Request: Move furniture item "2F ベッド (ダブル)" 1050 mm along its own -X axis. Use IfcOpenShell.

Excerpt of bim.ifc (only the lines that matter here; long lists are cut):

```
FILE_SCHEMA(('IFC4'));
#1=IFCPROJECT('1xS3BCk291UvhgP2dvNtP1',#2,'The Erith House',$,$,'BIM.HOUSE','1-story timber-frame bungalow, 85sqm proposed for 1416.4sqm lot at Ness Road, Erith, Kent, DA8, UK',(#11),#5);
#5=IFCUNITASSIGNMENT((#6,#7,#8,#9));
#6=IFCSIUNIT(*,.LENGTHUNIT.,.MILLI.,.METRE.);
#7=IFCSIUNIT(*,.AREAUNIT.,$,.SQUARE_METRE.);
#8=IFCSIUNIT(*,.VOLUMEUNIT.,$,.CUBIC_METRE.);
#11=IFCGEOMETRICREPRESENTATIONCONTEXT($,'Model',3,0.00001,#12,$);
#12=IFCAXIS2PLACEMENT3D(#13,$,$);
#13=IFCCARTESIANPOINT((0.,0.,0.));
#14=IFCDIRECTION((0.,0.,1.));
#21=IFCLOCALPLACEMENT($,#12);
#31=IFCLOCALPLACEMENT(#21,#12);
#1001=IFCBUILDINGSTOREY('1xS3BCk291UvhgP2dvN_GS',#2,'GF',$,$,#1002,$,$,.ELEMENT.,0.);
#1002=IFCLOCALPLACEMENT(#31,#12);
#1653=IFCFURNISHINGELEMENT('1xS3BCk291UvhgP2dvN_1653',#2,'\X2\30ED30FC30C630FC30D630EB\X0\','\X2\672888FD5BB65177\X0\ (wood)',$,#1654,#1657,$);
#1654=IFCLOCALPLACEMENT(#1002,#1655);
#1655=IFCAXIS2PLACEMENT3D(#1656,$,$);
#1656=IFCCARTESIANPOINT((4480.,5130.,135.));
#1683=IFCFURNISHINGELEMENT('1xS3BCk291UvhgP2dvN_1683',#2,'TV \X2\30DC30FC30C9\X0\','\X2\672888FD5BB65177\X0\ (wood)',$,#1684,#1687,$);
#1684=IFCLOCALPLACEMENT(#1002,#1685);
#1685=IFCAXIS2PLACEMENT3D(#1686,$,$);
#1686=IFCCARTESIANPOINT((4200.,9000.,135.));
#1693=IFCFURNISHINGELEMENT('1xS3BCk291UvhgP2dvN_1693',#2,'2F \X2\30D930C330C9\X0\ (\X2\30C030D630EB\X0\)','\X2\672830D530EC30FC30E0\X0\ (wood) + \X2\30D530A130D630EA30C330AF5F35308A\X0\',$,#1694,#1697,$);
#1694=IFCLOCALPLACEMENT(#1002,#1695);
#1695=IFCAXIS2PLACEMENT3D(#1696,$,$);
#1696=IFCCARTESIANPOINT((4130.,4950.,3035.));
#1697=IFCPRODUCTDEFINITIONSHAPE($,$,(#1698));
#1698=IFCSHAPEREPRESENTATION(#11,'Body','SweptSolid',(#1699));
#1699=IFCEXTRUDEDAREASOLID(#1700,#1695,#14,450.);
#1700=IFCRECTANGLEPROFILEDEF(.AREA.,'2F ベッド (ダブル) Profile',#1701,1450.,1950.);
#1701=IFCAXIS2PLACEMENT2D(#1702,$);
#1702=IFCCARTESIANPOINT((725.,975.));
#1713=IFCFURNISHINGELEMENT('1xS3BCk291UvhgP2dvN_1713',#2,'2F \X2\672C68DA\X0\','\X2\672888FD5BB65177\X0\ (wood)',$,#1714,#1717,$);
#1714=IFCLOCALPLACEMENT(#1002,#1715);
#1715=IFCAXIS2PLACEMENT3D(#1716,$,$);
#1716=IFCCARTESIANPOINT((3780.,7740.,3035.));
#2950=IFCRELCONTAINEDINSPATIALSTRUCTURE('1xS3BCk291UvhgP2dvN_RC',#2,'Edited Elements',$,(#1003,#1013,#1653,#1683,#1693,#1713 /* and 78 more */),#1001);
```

```python
import ifcopenshell
import ifcopenshell.api.geometry
import ifcopenshell.util.placement

model = ifcopenshell.open("bim.ifc")

item = model.by_id(1693)
matrix = ifcopenshell.util.placement.get_local_placement(item.ObjectPlacement)
matrix[:3, 3] -= matrix[:3, 0] * 1050.0
ifcopenshell.api.geometry.edit_object_placement(model, product=item, matrix=matrix, is_si=False)

print(ifcopenshell.util.placement.get_local_placement(item.ObjectPlacement).round(3) + 0.0)

model.write("bim_updated.ifc")
```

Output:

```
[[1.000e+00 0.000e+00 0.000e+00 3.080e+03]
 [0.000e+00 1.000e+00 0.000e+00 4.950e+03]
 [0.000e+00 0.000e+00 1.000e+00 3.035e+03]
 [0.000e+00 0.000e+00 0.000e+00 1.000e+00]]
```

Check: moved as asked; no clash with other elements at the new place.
